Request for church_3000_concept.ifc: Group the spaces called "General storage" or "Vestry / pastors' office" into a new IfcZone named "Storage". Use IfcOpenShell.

First a look at what the model holds.

```python
import ifcopenshell

model = ifcopenshell.open("church_3000_concept.ifc")
print(model.schema)
seen = {}
for space in model.by_type("IfcSpace"):
    seen[space.LongName] = seen.get(space.LongName, 0) + 1
for name, count in sorted(seen.items(), key=str):
    print(count, "x", name)
print("zones:", [z.Name for z in model.by_type("IfcZone")][:20])
```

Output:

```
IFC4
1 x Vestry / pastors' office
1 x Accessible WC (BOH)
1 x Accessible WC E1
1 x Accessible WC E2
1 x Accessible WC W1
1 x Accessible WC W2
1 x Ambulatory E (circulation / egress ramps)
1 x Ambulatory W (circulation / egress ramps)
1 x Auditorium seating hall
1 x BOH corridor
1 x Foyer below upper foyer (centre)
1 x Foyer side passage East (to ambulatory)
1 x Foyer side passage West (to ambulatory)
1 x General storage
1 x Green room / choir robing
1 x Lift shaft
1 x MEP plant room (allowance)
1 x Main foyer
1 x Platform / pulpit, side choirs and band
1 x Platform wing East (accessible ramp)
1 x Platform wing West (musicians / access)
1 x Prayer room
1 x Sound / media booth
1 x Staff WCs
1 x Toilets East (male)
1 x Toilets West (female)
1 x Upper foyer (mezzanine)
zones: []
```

```python
import ifcopenshell
import ifcopenshell.api.group
import ifcopenshell.api.root

model = ifcopenshell.open("church_3000_concept.ifc")

names = {"General storage", "Vestry / pastors' office"}
spaces = [s for s in model.by_type("IfcSpace") if s.LongName in names]

zone = ifcopenshell.api.root.create_entity(model, ifc_class="IfcZone", name="Storage")
ifcopenshell.api.group.assign_group(model, products=spaces, group=zone)
print(len(spaces), "spaces in", zone.Name)

model.write("church_3000_concept-out.ifc")
```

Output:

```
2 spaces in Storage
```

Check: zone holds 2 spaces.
